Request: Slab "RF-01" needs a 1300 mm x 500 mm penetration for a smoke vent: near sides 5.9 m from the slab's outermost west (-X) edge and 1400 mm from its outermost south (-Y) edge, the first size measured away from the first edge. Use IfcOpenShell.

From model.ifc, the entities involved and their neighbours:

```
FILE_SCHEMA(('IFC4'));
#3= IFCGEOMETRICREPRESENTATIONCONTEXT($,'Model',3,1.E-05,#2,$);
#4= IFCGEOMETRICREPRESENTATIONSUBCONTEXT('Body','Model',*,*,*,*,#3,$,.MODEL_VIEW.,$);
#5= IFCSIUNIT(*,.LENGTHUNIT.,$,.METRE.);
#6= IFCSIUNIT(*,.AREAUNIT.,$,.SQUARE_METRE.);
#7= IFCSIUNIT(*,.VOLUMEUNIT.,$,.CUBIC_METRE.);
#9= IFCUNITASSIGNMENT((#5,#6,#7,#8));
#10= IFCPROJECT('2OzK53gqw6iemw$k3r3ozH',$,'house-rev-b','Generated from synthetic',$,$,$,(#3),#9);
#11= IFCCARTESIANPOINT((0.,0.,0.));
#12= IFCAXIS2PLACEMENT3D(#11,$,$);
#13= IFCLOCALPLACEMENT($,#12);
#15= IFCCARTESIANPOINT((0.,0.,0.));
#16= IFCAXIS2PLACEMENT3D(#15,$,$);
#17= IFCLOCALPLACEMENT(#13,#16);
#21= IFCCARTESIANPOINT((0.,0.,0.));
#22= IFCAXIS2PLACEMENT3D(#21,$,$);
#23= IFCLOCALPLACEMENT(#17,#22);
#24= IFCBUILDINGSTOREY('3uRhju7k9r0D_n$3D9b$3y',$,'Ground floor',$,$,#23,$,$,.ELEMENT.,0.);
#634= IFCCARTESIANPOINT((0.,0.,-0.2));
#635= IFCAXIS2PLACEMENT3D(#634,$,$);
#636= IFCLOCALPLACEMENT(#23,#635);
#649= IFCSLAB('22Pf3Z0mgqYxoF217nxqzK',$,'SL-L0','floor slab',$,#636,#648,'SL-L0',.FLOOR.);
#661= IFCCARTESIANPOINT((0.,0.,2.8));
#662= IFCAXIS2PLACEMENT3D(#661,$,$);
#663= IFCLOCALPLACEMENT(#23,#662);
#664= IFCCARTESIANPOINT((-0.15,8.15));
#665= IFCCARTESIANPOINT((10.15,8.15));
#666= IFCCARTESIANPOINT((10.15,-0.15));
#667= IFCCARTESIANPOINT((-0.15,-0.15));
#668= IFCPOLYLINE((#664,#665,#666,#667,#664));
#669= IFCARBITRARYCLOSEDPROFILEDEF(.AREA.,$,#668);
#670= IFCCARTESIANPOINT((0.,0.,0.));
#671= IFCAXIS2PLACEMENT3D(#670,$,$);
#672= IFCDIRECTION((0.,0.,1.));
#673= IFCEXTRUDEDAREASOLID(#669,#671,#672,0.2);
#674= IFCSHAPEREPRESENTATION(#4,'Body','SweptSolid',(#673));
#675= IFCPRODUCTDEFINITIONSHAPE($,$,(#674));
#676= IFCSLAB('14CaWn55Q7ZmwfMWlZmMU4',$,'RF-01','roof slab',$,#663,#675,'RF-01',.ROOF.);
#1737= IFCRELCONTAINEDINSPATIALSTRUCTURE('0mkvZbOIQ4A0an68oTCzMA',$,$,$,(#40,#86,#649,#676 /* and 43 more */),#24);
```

```python
import numpy as np
import ifcopenshell
import ifcopenshell.api.feature
import ifcopenshell.api.geometry
import ifcopenshell.api.root
import ifcopenshell.geom
import ifcopenshell.util.placement
import ifcopenshell.util.representation
import ifcopenshell.util.shape
import ifcopenshell.util.unit

model = ifcopenshell.open("model.ifc")
unit_scale = ifcopenshell.util.unit.calculate_unit_scale(model)
settings = ifcopenshell.geom.settings()


def volume(element):
    """Net volume in cubic metres, openings subtracted."""
    shape = ifcopenshell.geom.create_shape(settings, element)
    return ifcopenshell.util.shape.get_volume(shape.geometry)


slab = model.by_guid("14CaWn55Q7ZmwfMWlZmMU4")
before = volume(slab)

# Extent in the slab's own axes, in metres. The edges named are its -X and -Y sides.
slab_shape = ifcopenshell.geom.create_shape(settings, slab)
vertices = ifcopenshell.util.shape.get_vertices(slab_shape.geometry)
x_min, y_min, bottom = vertices.min(axis=0)
top = vertices[:, 2].max()

opening = ifcopenshell.api.root.create_entity(model, ifc_class="IfcOpeningElement", name="Smoke vent opening", predefined_type="OPENING")
context = ifcopenshell.util.representation.get_context(model, "Model", "Body", "MODEL_VIEW")
width, depth = 1.3, 0.5
outline = [(0.0, 0.0), (width, 0.0), (width, depth), (0.0, depth), (0.0, 0.0)]
# Overshoot both faces by 50 mm so the cut is clean.
shape = ifcopenshell.api.geometry.add_slab_representation(
    model, context=context, depth=top - bottom + 0.1, polyline=outline
)
ifcopenshell.api.geometry.assign_representation(model, product=opening, representation=shape)

matrix = ifcopenshell.util.placement.get_local_placement(slab.ObjectPlacement)
matrix[:, 3] = matrix @ np.append(np.array([x_min + 5.9, y_min + 1.4, bottom - 0.05]) / unit_scale, 1.0)
ifcopenshell.api.geometry.edit_object_placement(model, product=opening, matrix=matrix, is_si=False)
ifcopenshell.api.feature.add_feature(model, feature=opening, element=slab)

after = volume(slab)

print(f"slab volume {before:.3f} -> {after:.3f} m3")

model.write("model_rev.ifc")
```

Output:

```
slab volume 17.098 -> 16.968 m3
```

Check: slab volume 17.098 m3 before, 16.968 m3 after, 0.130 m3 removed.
